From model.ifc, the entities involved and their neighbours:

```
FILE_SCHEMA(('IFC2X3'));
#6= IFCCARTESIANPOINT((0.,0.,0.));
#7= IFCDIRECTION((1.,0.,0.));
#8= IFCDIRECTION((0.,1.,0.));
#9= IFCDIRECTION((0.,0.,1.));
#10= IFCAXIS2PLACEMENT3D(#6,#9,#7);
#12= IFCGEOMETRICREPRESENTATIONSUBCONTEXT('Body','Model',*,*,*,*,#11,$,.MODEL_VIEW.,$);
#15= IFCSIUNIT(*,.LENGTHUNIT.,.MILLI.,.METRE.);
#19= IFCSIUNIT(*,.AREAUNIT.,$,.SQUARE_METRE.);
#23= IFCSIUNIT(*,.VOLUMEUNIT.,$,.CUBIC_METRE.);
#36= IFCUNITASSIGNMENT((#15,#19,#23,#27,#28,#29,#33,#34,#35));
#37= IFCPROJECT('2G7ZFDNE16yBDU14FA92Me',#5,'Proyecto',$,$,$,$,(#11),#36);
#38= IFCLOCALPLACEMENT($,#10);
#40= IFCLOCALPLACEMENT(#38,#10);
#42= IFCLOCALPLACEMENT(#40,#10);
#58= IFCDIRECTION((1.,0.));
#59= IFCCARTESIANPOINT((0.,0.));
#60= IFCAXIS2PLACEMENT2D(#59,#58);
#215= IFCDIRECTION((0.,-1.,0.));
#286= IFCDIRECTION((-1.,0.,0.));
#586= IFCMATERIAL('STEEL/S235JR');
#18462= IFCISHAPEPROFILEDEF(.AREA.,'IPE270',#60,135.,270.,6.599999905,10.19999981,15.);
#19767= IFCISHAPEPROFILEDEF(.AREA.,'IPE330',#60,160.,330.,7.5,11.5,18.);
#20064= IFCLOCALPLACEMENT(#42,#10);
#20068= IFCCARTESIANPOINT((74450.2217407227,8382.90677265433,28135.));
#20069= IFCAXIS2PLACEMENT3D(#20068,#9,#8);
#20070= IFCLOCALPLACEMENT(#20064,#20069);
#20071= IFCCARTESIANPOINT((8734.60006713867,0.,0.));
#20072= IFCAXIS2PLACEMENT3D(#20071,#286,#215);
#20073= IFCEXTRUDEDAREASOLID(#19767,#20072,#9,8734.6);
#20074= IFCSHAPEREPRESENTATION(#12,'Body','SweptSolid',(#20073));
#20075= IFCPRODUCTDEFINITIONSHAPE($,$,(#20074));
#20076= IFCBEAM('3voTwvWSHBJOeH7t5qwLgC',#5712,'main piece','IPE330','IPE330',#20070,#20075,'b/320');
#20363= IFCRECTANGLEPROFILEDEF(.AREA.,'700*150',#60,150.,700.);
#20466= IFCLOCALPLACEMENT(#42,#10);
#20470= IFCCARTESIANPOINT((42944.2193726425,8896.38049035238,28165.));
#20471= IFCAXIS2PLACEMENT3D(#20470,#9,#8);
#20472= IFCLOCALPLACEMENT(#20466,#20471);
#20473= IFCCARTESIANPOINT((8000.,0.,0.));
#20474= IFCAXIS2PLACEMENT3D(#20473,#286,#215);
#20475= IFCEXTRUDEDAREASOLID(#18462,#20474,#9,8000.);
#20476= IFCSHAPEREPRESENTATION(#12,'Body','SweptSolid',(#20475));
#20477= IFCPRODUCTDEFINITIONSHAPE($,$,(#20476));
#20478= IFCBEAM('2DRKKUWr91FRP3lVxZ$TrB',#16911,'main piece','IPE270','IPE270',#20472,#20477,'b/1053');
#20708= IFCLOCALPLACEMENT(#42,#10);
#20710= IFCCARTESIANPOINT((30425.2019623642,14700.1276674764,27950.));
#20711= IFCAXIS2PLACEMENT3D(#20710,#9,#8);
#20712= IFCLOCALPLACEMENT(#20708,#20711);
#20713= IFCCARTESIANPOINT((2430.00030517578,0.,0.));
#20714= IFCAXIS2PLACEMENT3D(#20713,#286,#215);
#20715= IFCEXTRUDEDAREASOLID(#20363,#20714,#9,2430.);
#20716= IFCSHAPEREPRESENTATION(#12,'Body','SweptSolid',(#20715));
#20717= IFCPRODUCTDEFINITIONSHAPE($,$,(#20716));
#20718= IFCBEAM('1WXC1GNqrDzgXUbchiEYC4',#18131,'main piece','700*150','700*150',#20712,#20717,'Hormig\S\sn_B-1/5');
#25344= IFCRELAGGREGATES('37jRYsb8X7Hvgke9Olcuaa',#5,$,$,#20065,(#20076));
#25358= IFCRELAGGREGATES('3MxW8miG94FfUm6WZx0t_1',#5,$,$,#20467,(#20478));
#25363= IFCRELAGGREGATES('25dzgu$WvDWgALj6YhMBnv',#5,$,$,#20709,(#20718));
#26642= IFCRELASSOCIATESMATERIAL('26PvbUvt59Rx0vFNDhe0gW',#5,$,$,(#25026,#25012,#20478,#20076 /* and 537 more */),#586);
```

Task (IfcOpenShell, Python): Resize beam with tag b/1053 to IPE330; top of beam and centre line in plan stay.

```python
import ifcopenshell
import ifcopenshell.util.element
import ifcopenshell.util.representation

model = ifcopenshell.open("model.ifc")

member = model.by_guid("2DRKKUWr91FRP3lVxZ$TrB")
source = next(p for p in model.by_type("IfcIShapeProfileDef") if p.ProfileName == "IPE330")

body = ifcopenshell.util.representation.get_representation(member, "Model", "Body")
solid = body.Items[0]
old_profile = solid.SweptArea

# Copy the section's sizes but keep this member's own profile position.
profile = ifcopenshell.util.element.copy(model, source)
# Profiles are centred, so shift by half the change in depth to hold the top.
shift = (old_profile.OverallDepth - profile.OverallDepth) / 2
x, y = old_profile.Position.Location.Coordinates
up = (0.0, 1.0)  # upwards, in the solid's own plane
location = model.createIfcCartesianPoint((x + up[0] * shift, y + up[1] * shift))
profile.Position = model.createIfcAxis2Placement2D(location, old_profile.Position.RefDirection)
solid.SweptArea = profile
if not model.get_total_inverses(old_profile):
    ifcopenshell.util.element.remove_deep2(model, old_profile)
member.Description = member.Description.replace("IPE270", "IPE330")
member.ObjectType = member.ObjectType.replace("IPE270", "IPE330")

print(solid.SweptArea)

model.write("model_rev.ifc")
```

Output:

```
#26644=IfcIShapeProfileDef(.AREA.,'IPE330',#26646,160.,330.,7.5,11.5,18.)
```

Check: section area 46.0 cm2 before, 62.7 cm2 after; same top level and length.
